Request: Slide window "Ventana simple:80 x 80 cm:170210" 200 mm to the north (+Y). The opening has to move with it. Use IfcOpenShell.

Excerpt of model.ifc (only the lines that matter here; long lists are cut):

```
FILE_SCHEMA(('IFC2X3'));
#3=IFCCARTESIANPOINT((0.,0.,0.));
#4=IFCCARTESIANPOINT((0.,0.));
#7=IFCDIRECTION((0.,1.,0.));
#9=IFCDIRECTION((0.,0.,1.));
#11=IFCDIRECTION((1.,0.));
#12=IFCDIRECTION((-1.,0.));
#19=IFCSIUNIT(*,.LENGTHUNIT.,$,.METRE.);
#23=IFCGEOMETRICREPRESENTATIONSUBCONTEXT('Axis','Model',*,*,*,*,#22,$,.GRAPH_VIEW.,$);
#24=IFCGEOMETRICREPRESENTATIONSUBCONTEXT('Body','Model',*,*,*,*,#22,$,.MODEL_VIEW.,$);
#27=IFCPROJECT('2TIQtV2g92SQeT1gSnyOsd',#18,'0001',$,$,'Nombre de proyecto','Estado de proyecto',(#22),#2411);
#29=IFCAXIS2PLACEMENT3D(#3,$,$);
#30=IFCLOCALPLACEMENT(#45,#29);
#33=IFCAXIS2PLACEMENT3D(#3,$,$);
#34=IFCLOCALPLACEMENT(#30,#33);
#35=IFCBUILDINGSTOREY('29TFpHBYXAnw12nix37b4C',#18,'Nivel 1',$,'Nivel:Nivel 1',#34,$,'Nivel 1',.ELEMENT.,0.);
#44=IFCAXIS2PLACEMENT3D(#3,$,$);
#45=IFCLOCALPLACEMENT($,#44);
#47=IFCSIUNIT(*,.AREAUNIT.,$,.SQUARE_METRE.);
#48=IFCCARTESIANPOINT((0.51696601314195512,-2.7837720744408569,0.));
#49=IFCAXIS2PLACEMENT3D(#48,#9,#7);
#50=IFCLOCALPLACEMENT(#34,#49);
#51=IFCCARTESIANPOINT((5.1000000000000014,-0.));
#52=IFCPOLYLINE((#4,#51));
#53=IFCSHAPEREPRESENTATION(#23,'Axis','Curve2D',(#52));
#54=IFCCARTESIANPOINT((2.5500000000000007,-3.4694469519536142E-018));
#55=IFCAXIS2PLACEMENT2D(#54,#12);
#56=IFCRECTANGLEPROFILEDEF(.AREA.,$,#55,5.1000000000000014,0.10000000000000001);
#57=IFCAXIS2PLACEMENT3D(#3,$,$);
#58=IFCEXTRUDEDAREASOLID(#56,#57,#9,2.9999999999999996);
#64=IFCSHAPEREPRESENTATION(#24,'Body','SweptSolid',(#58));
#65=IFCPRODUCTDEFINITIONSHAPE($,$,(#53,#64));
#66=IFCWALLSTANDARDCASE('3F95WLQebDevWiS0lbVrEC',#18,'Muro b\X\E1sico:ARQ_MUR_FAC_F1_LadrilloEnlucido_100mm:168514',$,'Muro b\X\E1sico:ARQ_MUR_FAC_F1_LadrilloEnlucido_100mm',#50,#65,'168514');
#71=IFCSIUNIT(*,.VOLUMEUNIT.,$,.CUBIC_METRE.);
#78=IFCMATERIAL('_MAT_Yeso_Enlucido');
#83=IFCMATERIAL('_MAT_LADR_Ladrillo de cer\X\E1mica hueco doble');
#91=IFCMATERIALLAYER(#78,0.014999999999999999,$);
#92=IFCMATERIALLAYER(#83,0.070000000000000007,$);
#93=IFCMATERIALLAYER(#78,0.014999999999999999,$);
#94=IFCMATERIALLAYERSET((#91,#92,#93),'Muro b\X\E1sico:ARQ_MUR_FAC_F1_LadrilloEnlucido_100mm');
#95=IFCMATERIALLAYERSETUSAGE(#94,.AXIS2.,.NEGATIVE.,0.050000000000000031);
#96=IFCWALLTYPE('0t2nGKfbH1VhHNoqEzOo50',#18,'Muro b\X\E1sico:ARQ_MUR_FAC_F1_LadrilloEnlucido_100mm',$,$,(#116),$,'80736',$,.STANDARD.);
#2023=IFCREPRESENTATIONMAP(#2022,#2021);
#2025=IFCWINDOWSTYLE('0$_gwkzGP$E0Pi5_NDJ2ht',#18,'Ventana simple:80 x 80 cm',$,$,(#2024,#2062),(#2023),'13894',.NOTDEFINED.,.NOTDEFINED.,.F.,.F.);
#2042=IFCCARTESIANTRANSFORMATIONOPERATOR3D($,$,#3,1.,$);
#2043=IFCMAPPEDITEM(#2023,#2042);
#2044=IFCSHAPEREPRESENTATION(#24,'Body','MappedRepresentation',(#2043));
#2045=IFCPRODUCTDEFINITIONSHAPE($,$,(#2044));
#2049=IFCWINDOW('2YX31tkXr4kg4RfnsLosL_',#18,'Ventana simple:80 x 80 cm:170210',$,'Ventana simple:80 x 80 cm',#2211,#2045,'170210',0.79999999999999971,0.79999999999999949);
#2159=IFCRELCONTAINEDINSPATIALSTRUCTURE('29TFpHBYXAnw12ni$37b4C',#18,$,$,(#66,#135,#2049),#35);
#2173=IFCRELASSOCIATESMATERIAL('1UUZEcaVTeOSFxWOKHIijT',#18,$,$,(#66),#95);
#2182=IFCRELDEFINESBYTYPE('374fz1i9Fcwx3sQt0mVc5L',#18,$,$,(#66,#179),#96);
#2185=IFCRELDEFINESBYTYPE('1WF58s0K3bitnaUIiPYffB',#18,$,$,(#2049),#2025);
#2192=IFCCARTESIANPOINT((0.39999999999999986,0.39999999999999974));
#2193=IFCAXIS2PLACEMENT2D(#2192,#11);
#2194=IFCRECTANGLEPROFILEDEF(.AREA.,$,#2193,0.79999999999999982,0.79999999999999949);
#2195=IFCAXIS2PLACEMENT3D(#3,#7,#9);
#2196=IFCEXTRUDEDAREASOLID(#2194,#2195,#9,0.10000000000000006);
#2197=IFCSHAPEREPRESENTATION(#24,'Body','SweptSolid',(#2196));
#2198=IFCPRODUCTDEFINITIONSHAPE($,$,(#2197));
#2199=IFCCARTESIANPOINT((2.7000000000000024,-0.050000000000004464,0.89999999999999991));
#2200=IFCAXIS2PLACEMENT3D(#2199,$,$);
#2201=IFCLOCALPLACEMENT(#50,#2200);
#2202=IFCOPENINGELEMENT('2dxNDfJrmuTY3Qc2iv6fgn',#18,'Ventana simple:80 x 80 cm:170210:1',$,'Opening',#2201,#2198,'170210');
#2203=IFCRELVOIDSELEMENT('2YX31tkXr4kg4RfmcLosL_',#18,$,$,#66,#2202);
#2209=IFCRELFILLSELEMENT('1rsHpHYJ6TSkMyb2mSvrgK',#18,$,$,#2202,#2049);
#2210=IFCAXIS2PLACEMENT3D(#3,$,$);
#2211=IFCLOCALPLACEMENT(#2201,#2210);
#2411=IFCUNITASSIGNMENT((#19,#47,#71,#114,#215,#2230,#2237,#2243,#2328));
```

```python
import ifcopenshell
import ifcopenshell.api.geometry
import ifcopenshell.util.placement

model = ifcopenshell.open("model.ifc")

window = model.by_id(2049)
opening = window.FillsVoids[0].RelatingOpeningElement
wall = opening.VoidsElements[0].RelatingBuildingElement

wall_matrix = ifcopenshell.util.placement.get_local_placement(wall.ObjectPlacement)
shift = wall_matrix[:3, 0] * 0.2
before = ifcopenshell.util.placement.get_local_placement(window.ObjectPlacement)[:3, 3].copy()

# The window is placed relative to its opening, so it follows when the opening moves.
matrix = ifcopenshell.util.placement.get_local_placement(opening.ObjectPlacement)
matrix[:3, 3] += shift
ifcopenshell.api.geometry.edit_object_placement(
    model, product=opening, matrix=matrix, is_si=False, should_transform_children=True
)

after = ifcopenshell.util.placement.get_local_placement(window.ObjectPlacement)[:3, 3]
print("window moved by", (after - before).round(3) + 0.0)

model.write("model-out.ifc")
```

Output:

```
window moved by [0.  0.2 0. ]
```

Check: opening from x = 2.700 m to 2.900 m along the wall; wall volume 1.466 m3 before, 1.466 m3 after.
